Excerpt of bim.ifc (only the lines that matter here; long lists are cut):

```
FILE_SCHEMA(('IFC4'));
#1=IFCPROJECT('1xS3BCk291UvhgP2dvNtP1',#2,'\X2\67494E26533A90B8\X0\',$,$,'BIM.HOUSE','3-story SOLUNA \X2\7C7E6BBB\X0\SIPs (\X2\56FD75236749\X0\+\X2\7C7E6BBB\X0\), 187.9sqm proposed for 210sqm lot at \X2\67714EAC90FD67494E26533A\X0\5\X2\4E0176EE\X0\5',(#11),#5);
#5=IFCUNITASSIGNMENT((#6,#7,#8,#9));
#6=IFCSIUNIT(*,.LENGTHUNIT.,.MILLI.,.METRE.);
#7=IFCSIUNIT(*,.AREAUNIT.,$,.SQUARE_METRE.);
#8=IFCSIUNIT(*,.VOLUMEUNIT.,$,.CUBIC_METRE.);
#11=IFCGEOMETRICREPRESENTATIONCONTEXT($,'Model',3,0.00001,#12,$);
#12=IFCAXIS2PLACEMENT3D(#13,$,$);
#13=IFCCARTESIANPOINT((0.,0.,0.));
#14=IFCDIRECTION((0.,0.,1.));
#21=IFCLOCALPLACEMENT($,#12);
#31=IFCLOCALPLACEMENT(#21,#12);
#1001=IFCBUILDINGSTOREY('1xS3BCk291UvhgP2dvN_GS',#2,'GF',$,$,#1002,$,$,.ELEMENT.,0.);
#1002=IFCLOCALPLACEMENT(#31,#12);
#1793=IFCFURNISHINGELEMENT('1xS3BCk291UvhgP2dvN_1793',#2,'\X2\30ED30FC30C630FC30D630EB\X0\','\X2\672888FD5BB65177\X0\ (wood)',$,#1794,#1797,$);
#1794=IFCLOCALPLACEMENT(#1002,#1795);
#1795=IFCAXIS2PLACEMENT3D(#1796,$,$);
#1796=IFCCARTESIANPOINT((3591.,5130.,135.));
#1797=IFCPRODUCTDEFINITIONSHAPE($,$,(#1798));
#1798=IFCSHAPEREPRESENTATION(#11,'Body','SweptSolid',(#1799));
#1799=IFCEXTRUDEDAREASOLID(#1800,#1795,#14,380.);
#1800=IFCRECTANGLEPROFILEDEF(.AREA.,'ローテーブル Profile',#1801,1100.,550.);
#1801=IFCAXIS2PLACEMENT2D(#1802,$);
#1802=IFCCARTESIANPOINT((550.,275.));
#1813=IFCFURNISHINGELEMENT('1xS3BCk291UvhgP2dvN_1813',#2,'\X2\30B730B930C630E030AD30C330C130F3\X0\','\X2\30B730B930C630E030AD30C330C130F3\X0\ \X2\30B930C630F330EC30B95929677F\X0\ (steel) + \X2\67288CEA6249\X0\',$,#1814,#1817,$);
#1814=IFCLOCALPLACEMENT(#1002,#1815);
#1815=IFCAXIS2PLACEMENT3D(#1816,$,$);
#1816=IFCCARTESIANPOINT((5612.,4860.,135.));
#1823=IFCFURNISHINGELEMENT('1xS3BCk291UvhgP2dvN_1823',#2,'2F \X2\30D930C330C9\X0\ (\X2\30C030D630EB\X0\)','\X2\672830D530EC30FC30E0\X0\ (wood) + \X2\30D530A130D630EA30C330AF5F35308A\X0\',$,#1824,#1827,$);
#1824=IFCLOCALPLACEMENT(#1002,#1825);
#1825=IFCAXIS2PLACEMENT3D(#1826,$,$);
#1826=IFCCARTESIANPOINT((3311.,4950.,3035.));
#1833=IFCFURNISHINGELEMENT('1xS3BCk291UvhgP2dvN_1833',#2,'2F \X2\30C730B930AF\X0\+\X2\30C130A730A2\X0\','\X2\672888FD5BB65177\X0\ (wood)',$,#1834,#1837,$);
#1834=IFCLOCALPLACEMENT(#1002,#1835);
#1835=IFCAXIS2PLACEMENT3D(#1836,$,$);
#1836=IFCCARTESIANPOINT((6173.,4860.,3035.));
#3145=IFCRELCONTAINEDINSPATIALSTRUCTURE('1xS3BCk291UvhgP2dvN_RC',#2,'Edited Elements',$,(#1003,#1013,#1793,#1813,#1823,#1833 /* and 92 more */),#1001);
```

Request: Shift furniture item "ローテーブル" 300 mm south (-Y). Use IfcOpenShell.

```python
import ifcopenshell
import ifcopenshell.api.geometry
import ifcopenshell.util.placement
import ifcopenshell.util.unit

model = ifcopenshell.open("bim.ifc")
unit_scale = ifcopenshell.util.unit.calculate_unit_scale(model)

item = model.by_guid("1xS3BCk291UvhgP2dvN_1793")
matrix = ifcopenshell.util.placement.get_local_placement(item.ObjectPlacement)
matrix[1, 3] -= 0.3 / unit_scale
ifcopenshell.api.geometry.edit_object_placement(model, product=item, matrix=matrix, is_si=False)

print(ifcopenshell.util.placement.get_local_placement(item.ObjectPlacement).round(3) + 0.0)

model.write("bim_edited.ifc")
```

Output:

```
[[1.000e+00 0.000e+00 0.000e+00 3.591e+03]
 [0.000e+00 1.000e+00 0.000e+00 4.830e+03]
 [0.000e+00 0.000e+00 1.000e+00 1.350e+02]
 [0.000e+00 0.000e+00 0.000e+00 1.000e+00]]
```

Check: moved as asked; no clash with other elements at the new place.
